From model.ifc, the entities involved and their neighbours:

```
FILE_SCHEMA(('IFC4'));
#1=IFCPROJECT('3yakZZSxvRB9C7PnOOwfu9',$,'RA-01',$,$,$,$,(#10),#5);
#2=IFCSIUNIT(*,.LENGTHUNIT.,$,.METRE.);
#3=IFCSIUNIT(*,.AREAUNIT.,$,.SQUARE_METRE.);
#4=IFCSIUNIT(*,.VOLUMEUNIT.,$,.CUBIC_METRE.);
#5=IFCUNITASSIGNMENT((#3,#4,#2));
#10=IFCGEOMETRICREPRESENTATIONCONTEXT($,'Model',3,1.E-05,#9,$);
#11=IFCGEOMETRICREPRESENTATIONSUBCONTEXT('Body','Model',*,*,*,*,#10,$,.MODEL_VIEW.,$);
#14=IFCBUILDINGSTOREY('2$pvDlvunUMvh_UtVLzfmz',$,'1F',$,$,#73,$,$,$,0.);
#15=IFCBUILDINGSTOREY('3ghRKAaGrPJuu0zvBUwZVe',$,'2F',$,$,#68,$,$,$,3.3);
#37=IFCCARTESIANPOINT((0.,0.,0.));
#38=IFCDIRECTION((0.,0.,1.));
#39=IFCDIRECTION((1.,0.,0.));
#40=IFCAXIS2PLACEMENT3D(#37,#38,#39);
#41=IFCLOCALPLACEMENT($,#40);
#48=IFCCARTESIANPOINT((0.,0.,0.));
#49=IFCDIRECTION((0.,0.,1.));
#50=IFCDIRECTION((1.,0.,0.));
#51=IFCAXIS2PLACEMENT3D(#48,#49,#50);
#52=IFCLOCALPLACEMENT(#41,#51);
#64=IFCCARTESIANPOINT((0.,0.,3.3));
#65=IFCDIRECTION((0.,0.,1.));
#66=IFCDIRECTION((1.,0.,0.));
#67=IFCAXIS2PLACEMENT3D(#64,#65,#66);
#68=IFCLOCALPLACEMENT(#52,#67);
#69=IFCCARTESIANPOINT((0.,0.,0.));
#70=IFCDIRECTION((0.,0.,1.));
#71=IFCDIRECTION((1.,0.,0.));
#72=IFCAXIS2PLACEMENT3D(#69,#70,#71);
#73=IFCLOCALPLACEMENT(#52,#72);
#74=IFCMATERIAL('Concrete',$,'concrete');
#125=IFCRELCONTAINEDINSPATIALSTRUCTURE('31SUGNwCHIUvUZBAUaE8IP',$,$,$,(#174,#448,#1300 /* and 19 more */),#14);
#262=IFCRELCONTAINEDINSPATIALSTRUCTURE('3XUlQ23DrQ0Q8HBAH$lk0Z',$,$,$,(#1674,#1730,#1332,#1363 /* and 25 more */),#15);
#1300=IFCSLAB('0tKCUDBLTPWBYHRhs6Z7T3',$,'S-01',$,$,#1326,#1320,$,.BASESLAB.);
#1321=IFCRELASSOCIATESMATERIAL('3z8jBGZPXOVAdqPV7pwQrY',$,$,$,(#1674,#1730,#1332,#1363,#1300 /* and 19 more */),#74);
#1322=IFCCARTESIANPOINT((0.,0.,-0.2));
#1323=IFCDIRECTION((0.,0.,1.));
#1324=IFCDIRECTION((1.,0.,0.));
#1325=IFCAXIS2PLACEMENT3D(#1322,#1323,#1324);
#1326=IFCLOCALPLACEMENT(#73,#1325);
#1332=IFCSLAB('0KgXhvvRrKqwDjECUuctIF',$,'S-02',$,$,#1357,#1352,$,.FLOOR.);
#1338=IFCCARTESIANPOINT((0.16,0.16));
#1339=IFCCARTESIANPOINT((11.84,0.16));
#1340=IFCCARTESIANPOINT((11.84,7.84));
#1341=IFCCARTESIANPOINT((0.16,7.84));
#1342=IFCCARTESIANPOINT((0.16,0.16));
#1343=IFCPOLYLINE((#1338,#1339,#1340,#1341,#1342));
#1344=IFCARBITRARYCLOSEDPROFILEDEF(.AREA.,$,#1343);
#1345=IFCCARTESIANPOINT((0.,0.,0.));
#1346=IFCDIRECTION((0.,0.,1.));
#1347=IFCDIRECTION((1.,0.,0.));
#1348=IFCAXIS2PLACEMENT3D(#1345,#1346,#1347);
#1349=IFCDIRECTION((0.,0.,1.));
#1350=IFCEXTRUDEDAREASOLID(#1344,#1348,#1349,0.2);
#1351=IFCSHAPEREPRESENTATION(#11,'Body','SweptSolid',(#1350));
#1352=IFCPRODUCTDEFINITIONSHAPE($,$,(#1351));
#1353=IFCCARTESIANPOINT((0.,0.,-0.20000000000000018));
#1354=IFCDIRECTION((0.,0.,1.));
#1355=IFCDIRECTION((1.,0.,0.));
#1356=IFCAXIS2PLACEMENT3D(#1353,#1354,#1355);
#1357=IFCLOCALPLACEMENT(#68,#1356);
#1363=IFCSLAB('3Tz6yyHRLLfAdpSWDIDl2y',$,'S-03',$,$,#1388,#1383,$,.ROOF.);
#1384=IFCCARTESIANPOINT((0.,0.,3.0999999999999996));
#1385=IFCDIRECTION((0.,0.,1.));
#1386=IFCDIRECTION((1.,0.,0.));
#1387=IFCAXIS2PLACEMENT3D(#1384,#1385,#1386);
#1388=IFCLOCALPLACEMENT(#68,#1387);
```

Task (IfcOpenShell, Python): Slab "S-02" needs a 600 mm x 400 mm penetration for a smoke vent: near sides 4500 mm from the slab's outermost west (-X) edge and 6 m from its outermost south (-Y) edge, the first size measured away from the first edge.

```python
import numpy as np
import ifcopenshell
import ifcopenshell.api.feature
import ifcopenshell.api.geometry
import ifcopenshell.api.root
import ifcopenshell.geom
import ifcopenshell.util.placement
import ifcopenshell.util.representation
import ifcopenshell.util.shape
import ifcopenshell.util.unit

model = ifcopenshell.open("model.ifc")
unit_scale = ifcopenshell.util.unit.calculate_unit_scale(model)
settings = ifcopenshell.geom.settings()


def volume(element):
    """Net volume in cubic metres, openings subtracted."""
    shape = ifcopenshell.geom.create_shape(settings, element)
    return ifcopenshell.util.shape.get_volume(shape.geometry)


slab = model.by_guid("0KgXhvvRrKqwDjECUuctIF")
before = volume(slab)

# Extent in the slab's own axes, in metres. The edges named are its -X and -Y sides.
slab_shape = ifcopenshell.geom.create_shape(settings, slab)
vertices = ifcopenshell.util.shape.get_vertices(slab_shape.geometry)
x_min, y_min, bottom = vertices.min(axis=0)
top = vertices[:, 2].max()

opening = ifcopenshell.api.root.create_entity(model, ifc_class="IfcOpeningElement", name="Smoke vent opening", predefined_type="OPENING")
context = ifcopenshell.util.representation.get_context(model, "Model", "Body", "MODEL_VIEW")
width, depth = 0.6, 0.4
outline = [(0.0, 0.0), (width, 0.0), (width, depth), (0.0, depth), (0.0, 0.0)]
# Overshoot both faces by 50 mm so the cut is clean.
shape = ifcopenshell.api.geometry.add_slab_representation(
    model, context=context, depth=top - bottom + 0.1, polyline=outline
)
ifcopenshell.api.geometry.assign_representation(model, product=opening, representation=shape)

matrix = ifcopenshell.util.placement.get_local_placement(slab.ObjectPlacement)
matrix[:, 3] = matrix @ np.append(np.array([x_min + 4.5, y_min + 6, bottom - 0.05]) / unit_scale, 1.0)
ifcopenshell.api.geometry.edit_object_placement(model, product=opening, matrix=matrix, is_si=False)
ifcopenshell.api.feature.add_feature(model, feature=opening, element=slab)

after = volume(slab)

print(f"slab volume {before:.3f} -> {after:.3f} m3")

model.write("model_v2.ifc")
```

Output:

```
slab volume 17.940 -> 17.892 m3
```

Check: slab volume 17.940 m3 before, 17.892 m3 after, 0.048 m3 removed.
